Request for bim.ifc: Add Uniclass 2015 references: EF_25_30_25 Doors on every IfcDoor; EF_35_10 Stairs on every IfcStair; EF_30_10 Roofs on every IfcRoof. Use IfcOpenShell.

First a look at what the model holds.

```python
import ifcopenshell

model = ifcopenshell.open("bim.ifc")
print(model.schema)
print("classifications:", [c.Name for c in model.by_type("IfcClassification")])
for ifc_class in ("IfcDoor", "IfcRoof", "IfcStair", "IfcWall", "IfcWindow"):
    print(ifc_class, len(model.by_type(ifc_class)))
```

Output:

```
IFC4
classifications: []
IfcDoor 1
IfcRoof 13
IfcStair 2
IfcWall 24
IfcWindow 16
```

```python
import ifcopenshell
import ifcopenshell.api.classification

model = ifcopenshell.open("bim.ifc")

system = ifcopenshell.api.classification.add_classification(model, classification="Uniclass 2015")

codes = {
    "IfcDoor": ("EF_25_30_25", "Doors"),
    "IfcStair": ("EF_35_10", "Stairs"),
    "IfcRoof": ("EF_30_10", "Roofs"),
}
for ifc_class, (code, name) in codes.items():
    products = model.by_type(ifc_class)
    ifcopenshell.api.classification.add_reference(
        model, products=products, classification=system, identification=code, name=name
    )
    print(code, len(products))

model.write("bim_edited.ifc")
```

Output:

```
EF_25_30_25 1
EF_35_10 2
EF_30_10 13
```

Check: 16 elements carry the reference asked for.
